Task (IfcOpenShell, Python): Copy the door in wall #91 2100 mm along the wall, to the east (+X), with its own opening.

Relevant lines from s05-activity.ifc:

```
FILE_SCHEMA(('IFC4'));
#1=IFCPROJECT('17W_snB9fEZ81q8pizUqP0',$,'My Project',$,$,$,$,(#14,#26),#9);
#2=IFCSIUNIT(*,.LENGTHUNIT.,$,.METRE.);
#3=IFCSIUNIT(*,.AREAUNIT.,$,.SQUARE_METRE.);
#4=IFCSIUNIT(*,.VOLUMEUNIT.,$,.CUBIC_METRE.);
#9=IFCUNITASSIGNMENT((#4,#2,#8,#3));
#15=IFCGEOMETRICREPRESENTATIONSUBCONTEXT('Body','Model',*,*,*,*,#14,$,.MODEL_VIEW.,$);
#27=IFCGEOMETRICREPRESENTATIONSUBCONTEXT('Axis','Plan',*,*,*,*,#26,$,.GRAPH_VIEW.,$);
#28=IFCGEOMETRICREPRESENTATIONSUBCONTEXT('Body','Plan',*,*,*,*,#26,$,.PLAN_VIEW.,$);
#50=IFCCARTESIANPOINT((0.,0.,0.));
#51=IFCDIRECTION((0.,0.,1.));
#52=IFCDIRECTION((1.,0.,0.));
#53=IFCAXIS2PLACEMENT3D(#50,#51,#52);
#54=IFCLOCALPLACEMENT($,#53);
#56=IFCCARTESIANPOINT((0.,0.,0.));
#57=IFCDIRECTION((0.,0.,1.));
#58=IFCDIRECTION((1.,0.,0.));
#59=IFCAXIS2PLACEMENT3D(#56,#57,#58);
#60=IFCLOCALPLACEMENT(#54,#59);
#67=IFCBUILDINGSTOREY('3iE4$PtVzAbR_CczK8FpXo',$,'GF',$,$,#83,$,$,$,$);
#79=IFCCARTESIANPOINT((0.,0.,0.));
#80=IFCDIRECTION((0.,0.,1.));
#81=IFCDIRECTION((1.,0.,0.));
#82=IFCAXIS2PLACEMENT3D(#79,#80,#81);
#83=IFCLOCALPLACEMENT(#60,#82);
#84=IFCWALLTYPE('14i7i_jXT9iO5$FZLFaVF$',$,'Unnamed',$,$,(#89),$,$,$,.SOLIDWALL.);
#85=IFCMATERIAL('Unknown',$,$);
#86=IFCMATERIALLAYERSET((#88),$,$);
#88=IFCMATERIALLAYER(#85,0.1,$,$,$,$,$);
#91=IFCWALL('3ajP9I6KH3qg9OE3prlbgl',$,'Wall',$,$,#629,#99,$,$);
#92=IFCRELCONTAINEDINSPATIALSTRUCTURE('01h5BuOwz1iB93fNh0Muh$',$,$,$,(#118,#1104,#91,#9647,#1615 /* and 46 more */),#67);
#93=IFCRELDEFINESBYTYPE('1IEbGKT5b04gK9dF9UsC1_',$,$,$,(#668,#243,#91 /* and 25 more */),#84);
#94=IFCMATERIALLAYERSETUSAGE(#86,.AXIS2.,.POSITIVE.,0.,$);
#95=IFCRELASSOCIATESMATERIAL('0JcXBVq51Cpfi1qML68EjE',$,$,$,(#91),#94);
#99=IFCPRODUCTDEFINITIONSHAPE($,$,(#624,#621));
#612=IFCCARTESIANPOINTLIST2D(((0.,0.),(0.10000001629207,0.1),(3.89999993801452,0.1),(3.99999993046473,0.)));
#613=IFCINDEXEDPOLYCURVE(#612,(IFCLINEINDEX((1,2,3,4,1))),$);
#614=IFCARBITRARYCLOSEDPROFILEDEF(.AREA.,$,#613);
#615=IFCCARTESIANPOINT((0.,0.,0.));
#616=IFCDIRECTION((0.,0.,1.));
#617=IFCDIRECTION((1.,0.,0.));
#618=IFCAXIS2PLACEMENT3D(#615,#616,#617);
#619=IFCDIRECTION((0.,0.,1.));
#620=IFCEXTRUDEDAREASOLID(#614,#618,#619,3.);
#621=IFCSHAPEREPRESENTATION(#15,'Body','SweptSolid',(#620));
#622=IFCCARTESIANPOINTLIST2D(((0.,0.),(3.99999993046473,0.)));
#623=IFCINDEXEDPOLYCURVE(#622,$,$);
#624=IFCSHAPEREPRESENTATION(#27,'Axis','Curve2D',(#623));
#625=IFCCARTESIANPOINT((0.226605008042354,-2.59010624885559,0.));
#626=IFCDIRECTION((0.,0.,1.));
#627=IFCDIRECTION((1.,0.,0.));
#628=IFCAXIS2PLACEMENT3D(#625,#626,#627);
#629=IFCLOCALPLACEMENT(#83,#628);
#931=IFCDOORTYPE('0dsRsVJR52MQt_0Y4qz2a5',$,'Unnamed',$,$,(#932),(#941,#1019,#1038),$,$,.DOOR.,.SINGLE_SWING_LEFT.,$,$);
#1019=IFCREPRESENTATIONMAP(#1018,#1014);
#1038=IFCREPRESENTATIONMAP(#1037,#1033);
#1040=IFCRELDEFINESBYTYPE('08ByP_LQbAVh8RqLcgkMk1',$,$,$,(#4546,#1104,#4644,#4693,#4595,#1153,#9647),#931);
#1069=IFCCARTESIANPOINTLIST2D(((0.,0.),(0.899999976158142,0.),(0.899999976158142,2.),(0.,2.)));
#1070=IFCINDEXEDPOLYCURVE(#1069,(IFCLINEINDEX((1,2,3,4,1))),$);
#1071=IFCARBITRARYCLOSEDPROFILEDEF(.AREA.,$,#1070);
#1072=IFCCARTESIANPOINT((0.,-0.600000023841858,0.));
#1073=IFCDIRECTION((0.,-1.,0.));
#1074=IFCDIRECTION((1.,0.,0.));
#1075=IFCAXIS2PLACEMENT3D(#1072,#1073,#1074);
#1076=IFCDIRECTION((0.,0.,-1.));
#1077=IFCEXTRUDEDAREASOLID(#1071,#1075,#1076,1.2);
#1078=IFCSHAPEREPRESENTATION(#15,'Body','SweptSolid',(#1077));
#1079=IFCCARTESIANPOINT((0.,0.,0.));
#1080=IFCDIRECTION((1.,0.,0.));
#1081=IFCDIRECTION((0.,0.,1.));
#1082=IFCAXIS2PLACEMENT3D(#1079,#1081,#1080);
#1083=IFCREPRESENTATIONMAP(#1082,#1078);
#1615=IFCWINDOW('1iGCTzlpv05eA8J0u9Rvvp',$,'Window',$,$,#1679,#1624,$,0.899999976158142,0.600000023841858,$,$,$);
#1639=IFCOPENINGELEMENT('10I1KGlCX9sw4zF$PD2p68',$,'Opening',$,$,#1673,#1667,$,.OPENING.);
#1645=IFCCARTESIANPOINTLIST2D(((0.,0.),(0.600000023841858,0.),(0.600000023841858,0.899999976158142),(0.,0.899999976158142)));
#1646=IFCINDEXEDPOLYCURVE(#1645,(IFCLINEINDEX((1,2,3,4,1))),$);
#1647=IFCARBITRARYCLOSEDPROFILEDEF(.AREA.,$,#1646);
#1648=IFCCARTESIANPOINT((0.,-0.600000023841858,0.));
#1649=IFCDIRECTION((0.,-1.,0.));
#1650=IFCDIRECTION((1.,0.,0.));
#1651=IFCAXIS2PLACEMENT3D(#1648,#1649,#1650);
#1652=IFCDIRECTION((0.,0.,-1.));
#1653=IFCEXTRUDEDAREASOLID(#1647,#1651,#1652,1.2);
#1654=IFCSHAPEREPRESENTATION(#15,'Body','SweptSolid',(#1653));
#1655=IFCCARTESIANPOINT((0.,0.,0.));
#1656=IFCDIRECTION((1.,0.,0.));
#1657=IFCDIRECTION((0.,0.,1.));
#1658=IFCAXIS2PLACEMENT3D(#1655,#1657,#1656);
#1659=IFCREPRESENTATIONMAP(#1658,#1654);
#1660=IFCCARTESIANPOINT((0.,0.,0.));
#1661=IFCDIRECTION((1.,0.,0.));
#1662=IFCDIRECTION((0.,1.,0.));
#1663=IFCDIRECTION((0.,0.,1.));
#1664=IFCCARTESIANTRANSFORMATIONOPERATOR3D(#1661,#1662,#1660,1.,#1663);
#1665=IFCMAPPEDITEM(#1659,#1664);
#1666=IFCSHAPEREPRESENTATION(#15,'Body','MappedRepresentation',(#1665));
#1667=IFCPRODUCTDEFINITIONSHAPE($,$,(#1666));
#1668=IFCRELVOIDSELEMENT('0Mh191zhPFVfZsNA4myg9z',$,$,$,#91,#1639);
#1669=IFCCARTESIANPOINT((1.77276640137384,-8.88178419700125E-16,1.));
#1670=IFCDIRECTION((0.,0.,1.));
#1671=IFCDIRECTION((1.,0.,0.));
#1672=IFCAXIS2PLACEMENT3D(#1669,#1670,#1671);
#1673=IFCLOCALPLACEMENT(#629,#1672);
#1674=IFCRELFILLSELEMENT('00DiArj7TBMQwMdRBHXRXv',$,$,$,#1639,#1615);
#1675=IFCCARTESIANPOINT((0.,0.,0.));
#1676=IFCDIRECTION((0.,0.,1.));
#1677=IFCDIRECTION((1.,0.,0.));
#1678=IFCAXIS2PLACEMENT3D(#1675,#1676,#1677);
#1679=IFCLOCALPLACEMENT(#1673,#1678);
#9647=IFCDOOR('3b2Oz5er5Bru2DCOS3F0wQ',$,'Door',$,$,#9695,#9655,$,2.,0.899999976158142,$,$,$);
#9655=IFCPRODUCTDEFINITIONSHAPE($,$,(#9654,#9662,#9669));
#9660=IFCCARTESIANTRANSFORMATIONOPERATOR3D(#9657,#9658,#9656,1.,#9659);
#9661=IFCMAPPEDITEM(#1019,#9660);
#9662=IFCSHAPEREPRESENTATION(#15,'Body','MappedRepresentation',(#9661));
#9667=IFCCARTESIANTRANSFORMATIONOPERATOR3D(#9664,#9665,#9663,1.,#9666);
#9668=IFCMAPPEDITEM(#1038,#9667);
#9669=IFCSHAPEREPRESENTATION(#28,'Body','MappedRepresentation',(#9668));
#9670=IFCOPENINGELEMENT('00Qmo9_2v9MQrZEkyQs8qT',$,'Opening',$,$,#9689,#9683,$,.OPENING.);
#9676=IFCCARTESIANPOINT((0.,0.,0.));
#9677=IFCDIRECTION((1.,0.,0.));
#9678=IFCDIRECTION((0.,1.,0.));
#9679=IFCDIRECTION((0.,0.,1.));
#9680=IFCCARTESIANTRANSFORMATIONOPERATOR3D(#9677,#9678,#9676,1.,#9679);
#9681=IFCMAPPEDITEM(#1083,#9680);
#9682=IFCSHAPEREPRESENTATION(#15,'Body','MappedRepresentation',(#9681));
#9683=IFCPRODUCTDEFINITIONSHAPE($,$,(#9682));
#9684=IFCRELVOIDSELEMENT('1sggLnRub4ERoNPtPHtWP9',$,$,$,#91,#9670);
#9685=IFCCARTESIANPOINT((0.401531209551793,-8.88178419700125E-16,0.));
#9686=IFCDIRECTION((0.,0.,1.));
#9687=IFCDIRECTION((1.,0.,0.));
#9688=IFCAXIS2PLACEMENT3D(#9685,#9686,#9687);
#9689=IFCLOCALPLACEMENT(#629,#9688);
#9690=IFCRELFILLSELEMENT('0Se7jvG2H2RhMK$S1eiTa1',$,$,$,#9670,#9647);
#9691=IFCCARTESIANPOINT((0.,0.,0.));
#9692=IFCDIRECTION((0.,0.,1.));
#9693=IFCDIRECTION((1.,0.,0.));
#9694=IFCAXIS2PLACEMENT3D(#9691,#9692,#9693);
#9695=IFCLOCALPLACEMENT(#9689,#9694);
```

```python
import ifcopenshell
import ifcopenshell.api.feature
import ifcopenshell.api.geometry
import ifcopenshell.api.root
import ifcopenshell.geom
import ifcopenshell.util.element
import ifcopenshell.util.placement
import ifcopenshell.util.shape

model = ifcopenshell.open("s05-activity.ifc")
settings = ifcopenshell.geom.settings()


def volume(element):
    """Net volume in cubic metres, openings subtracted."""
    shape = ifcopenshell.geom.create_shape(settings, element)
    return ifcopenshell.util.shape.get_volume(shape.geometry)


door = model.by_id(9647)
opening = door.FillsVoids[0].RelatingOpeningElement
wall = opening.VoidsElements[0].RelatingBuildingElement
before = volume(wall)
shift = ifcopenshell.util.placement.get_local_placement(wall.ObjectPlacement)[:3, 0] * 2.1

# copy_class copies the void relationship, type, container and properties, but no geometry.
new_opening = ifcopenshell.api.root.copy_class(model, product=opening)
new_opening.Representation = ifcopenshell.util.element.copy_deep(
    model, opening.Representation, exclude=["IfcGeometricRepresentationContext", "IfcRepresentationMap"]
)
new_door = ifcopenshell.api.root.copy_class(model, product=door)
new_door.Representation = ifcopenshell.util.element.copy_deep(
    model, door.Representation, exclude=["IfcGeometricRepresentationContext", "IfcRepresentationMap"]
)
ifcopenshell.api.feature.add_filling(model, opening=new_opening, element=new_door)

for old, new in ((opening, new_opening), (door, new_door)):
    matrix = ifcopenshell.util.placement.get_local_placement(old.ObjectPlacement)
    matrix[:3, 3] += shift
    ifcopenshell.api.geometry.edit_object_placement(model, product=new, matrix=matrix, is_si=False)

after = volume(wall)

print(f"wall volume {before:.3f} -> {after:.3f} m3")

model.write("s05-activity_edited.ifc")
```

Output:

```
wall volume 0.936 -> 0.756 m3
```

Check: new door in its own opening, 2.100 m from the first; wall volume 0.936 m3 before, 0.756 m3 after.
